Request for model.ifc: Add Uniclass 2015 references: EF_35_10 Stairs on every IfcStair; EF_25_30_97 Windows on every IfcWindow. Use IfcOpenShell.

First a look at what the model holds.

```python
import ifcopenshell

model = ifcopenshell.open("model.ifc")
print(model.schema)
print("classifications:", [c.Name for c in model.by_type("IfcClassification")])
for ifc_class in ("IfcDoor", "IfcRoof", "IfcStair", "IfcWall", "IfcWindow"):
    print(ifc_class, len(model.by_type(ifc_class)))
```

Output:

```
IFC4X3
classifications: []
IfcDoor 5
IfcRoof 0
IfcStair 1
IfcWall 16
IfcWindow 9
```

```python
import ifcopenshell
import ifcopenshell.api.classification

model = ifcopenshell.open("model.ifc")

system = ifcopenshell.api.classification.add_classification(model, classification="Uniclass 2015")

codes = {
    "IfcStair": ("EF_35_10", "Stairs"),
    "IfcWindow": ("EF_25_30_97", "Windows"),
}
for ifc_class, (code, name) in codes.items():
    products = model.by_type(ifc_class)
    ifcopenshell.api.classification.add_reference(
        model, products=products, classification=system, identification=code, name=name
    )
    print(code, len(products))

model.write("model_v2.ifc")
```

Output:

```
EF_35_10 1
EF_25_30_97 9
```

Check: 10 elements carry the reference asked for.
